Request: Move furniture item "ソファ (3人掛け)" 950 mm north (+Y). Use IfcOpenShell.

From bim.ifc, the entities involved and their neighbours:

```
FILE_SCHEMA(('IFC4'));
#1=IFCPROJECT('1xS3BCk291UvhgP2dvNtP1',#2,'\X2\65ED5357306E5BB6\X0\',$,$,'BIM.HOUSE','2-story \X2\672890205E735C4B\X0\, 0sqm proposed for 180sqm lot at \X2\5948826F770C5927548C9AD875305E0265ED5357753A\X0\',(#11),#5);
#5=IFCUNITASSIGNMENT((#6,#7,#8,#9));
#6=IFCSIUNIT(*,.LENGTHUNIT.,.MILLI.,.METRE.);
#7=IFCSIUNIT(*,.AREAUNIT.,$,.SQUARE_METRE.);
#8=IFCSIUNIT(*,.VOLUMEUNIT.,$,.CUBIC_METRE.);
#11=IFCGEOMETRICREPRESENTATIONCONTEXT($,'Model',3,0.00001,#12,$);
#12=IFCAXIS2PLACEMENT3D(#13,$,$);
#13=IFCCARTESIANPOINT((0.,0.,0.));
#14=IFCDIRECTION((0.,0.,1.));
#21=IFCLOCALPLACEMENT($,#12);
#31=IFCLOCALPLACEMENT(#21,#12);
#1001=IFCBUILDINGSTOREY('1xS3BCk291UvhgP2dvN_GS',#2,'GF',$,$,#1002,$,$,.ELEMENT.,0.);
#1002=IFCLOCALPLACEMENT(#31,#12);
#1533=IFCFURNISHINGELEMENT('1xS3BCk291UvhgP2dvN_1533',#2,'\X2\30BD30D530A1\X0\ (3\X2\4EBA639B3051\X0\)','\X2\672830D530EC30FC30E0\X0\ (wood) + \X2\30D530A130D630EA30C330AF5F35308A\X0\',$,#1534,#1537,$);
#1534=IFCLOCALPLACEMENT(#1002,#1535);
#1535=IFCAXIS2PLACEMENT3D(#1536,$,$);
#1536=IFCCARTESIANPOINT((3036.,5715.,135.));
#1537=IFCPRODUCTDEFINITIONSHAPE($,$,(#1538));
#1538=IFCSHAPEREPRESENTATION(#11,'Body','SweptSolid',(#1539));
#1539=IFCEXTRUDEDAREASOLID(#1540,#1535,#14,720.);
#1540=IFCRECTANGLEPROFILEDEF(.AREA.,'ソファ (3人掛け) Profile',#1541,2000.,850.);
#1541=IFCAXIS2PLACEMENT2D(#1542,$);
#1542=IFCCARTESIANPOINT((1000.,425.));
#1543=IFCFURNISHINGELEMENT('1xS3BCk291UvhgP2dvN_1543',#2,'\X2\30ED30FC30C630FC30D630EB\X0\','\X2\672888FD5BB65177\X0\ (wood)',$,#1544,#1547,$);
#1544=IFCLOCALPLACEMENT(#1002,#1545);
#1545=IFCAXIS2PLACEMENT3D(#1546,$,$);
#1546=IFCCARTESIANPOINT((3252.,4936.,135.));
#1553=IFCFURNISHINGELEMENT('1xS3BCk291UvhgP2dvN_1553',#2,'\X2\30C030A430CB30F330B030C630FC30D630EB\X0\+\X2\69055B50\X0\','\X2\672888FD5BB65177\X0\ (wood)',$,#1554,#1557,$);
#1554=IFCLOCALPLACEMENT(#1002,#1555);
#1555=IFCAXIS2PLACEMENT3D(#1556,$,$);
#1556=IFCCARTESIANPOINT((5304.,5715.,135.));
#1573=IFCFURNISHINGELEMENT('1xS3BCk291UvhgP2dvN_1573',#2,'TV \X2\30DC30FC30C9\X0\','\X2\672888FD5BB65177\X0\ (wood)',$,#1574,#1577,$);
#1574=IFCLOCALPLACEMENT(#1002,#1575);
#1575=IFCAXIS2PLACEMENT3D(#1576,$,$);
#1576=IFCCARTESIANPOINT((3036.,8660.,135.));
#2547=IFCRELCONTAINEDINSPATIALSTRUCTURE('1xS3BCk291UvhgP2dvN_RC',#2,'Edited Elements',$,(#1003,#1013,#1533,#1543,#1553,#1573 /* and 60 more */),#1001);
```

```python
import ifcopenshell
import ifcopenshell.api.geometry
import ifcopenshell.util.placement
import ifcopenshell.util.unit

model = ifcopenshell.open("bim.ifc")
unit_scale = ifcopenshell.util.unit.calculate_unit_scale(model)

item = model.by_id(1533)
matrix = ifcopenshell.util.placement.get_local_placement(item.ObjectPlacement)
matrix[1, 3] += 0.95 / unit_scale
ifcopenshell.api.geometry.edit_object_placement(model, product=item, matrix=matrix, is_si=False)

print(ifcopenshell.util.placement.get_local_placement(item.ObjectPlacement).round(3) + 0.0)

model.write("bim_v2.ifc")
```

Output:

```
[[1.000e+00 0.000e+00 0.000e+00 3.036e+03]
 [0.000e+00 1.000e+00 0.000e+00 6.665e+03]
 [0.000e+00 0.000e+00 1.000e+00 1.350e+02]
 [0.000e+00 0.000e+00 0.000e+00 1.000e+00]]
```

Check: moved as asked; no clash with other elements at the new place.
